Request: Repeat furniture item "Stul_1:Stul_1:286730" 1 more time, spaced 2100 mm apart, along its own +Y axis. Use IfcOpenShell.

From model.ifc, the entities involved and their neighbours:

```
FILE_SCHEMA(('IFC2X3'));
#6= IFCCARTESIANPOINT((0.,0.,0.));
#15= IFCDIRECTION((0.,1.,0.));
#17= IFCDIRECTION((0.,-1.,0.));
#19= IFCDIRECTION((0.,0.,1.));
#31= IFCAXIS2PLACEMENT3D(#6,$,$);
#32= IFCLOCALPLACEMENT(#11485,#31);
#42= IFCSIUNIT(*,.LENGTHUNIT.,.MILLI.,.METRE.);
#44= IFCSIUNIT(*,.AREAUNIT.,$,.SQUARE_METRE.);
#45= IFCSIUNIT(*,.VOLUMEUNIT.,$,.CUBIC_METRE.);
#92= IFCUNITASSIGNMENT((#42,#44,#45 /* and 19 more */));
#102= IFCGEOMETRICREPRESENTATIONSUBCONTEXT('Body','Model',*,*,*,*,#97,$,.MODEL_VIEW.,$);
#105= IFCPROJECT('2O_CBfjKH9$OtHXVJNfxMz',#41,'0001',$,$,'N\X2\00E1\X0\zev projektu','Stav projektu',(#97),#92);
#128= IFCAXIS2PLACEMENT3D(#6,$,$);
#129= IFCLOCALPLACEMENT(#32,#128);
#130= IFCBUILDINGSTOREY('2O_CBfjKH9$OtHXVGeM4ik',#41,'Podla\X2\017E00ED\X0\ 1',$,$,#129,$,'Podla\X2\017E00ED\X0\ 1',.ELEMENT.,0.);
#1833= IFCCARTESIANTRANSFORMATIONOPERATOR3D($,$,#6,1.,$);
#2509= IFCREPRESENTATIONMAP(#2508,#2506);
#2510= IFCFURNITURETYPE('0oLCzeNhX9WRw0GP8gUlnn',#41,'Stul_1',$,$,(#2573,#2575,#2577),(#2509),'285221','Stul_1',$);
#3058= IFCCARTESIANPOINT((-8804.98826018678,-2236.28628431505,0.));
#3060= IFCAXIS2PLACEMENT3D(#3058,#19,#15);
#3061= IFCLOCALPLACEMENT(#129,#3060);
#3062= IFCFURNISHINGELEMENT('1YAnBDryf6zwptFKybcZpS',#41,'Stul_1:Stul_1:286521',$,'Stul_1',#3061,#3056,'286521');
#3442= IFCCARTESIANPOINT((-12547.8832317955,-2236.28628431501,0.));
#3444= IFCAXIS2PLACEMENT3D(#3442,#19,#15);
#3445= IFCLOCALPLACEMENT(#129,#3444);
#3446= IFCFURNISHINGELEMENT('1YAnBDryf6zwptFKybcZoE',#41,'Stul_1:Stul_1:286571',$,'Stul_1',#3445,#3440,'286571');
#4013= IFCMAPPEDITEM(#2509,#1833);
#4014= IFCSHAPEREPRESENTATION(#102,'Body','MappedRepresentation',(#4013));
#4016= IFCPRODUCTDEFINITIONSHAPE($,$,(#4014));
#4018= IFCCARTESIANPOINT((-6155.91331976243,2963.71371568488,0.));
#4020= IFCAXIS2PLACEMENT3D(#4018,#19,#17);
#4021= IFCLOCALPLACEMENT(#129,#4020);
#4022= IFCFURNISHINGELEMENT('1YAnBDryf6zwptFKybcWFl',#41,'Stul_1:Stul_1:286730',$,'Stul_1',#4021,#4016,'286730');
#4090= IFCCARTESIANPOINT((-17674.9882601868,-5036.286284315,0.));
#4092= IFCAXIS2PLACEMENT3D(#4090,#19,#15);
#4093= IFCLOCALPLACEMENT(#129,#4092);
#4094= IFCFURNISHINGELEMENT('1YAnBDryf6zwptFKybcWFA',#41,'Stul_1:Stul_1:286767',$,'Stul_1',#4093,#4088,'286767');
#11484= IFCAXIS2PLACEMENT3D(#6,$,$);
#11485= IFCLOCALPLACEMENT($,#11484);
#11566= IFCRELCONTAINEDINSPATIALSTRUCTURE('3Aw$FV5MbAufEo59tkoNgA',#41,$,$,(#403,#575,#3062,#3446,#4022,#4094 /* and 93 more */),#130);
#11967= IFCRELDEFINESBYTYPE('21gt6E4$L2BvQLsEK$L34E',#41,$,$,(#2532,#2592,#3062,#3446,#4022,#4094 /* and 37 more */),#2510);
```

```python
import ifcopenshell
import ifcopenshell.api.geometry
import ifcopenshell.api.root
import ifcopenshell.util.element
import ifcopenshell.util.placement
import ifcopenshell.util.unit

model = ifcopenshell.open("model.ifc")
unit_scale = ifcopenshell.util.unit.calculate_unit_scale(model)


def reuse_history(source, copy):
    """copy_class also copies each property set's owner history, people and application; keep the originals."""
    for rel in copy.IsDefinedBy:
        if rel.is_a("IfcRelDefinesByProperties") and (history := rel.RelatingPropertyDefinition.OwnerHistory):
            rel.RelatingPropertyDefinition.OwnerHistory = source.OwnerHistory
            ifcopenshell.util.element.remove_deep2(model, history)


source = model.by_id(4022)
base = ifcopenshell.util.placement.get_local_placement(source.ObjectPlacement)
step = base[:3, 1] * 2.1 / unit_scale

for i in range(1, 2):
    copy = ifcopenshell.api.root.copy_class(model, product=source)
    copy.Representation = ifcopenshell.util.element.copy_deep(
        model, source.Representation, exclude=["IfcGeometricRepresentationContext", "IfcRepresentationMap"]
    )
    copy.Name = "Stul_1:Stul_1"
    copy.Tag = None
    reuse_history(source, copy)
    matrix = base.copy()
    matrix[:3, 3] += i * step
    print("added at", matrix[:3, 3].round(3) + 0.0)
    ifcopenshell.api.geometry.edit_object_placement(model, product=copy, matrix=matrix, is_si=False)

model.write("model_updated.ifc")
```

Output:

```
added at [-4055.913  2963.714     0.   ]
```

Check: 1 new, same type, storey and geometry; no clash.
